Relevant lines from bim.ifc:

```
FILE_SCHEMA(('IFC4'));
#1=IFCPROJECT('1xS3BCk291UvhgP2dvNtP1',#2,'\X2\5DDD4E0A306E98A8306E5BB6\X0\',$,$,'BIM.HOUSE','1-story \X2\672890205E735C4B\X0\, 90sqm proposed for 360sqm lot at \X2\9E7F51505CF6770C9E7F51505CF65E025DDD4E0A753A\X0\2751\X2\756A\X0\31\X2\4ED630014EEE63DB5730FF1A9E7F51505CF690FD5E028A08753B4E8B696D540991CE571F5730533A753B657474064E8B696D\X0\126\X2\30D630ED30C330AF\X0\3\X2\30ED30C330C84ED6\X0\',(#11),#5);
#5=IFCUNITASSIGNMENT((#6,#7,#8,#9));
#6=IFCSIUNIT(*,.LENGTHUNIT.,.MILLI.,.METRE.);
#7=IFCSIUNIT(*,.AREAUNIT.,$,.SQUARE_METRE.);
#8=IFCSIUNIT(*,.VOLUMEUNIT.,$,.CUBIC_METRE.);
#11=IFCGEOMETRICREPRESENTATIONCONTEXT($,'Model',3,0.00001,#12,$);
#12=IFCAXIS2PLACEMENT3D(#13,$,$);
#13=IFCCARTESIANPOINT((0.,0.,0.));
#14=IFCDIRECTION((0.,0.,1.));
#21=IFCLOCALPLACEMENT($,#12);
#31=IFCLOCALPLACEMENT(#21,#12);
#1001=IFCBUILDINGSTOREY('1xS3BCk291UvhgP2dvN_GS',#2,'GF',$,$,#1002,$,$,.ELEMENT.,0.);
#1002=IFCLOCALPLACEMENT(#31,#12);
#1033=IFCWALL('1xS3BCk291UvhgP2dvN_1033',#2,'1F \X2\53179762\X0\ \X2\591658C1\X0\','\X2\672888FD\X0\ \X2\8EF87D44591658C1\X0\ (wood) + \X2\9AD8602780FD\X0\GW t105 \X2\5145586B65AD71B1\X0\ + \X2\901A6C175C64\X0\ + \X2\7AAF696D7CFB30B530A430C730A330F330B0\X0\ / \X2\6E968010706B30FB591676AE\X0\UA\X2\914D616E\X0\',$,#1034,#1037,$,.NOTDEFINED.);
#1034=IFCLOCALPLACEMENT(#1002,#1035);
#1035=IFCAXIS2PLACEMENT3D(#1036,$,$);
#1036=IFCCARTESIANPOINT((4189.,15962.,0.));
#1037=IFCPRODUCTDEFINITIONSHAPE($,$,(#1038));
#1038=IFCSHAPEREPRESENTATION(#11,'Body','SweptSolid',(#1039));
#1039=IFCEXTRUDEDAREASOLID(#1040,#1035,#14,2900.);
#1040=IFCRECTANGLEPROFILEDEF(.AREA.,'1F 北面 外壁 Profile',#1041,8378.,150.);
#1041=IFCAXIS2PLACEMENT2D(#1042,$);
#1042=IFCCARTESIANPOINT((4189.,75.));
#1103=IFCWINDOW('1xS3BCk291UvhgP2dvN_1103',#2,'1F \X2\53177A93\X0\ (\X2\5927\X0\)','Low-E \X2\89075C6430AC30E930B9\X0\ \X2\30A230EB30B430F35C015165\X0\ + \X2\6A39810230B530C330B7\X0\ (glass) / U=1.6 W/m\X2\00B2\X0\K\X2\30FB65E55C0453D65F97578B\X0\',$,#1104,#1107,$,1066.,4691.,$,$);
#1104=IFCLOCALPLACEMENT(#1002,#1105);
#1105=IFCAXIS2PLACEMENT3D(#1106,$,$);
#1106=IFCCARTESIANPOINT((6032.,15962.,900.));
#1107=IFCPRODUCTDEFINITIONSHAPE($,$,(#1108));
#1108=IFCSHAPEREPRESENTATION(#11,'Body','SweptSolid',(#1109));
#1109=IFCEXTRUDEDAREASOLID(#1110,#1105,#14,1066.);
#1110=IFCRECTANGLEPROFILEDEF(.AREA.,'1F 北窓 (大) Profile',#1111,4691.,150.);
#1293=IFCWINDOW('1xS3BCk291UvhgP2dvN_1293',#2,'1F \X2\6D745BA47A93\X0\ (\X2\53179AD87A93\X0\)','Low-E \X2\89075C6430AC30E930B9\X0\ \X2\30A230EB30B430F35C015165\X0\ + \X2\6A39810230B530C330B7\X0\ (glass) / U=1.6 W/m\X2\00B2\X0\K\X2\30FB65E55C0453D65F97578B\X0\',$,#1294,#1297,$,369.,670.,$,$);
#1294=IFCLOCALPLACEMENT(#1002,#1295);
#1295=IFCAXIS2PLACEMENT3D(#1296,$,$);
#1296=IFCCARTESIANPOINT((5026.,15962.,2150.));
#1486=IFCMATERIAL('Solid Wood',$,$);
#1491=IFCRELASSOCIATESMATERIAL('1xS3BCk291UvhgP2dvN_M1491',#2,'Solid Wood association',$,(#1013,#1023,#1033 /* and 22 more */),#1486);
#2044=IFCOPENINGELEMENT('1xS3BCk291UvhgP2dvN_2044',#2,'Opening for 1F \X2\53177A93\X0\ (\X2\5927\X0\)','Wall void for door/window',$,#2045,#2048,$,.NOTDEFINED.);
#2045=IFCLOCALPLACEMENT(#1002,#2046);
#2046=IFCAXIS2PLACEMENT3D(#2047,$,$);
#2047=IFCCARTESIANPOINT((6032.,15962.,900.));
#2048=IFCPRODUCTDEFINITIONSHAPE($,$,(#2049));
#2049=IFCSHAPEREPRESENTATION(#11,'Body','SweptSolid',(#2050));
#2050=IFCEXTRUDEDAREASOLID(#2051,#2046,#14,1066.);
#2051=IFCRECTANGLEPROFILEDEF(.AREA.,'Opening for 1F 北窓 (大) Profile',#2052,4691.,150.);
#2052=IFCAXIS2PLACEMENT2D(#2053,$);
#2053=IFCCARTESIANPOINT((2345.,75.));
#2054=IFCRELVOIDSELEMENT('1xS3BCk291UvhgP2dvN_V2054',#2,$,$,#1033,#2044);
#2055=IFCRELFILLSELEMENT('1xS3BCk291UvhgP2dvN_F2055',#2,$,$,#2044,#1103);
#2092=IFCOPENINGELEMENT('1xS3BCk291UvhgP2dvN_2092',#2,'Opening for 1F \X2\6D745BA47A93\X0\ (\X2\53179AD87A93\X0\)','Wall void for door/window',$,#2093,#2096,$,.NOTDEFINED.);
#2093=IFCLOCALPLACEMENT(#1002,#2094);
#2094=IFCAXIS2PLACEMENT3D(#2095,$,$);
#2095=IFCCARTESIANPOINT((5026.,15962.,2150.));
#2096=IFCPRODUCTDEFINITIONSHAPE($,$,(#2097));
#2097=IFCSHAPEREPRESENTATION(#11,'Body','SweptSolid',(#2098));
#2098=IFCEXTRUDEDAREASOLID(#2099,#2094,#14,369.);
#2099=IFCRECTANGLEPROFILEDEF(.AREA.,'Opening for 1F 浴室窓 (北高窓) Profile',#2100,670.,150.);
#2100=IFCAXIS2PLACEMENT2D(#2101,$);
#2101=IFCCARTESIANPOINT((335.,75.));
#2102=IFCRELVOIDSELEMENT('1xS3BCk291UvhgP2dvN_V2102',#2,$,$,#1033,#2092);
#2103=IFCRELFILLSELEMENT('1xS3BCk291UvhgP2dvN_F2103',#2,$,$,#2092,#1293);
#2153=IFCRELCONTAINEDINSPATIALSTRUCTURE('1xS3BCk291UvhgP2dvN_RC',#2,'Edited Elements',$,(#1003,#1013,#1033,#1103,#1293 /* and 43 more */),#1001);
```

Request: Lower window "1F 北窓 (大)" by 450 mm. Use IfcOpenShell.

```python
import numpy as np
import ifcopenshell
import ifcopenshell.api.geometry
import ifcopenshell.util.placement
import ifcopenshell.util.unit

model = ifcopenshell.open("bim.ifc")
unit_scale = ifcopenshell.util.unit.calculate_unit_scale(model)

window = model.by_guid("1xS3BCk291UvhgP2dvN_1103")
opening = window.FillsVoids[0].RelatingOpeningElement
dz = -450.0

shift = np.array([0.0, 0.0, dz])
# The window is not placed relative to its opening, so move both.
for product in (opening, window):
    matrix = ifcopenshell.util.placement.get_local_placement(product.ObjectPlacement)
    matrix[:3, 3] += shift
    ifcopenshell.api.geometry.edit_object_placement(model, product=product, matrix=matrix, is_si=False)

print(f"moved by {dz * unit_scale:+.3f} m")

model.write("bim-out.ifc")
```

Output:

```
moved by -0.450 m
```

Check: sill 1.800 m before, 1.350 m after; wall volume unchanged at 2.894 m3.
